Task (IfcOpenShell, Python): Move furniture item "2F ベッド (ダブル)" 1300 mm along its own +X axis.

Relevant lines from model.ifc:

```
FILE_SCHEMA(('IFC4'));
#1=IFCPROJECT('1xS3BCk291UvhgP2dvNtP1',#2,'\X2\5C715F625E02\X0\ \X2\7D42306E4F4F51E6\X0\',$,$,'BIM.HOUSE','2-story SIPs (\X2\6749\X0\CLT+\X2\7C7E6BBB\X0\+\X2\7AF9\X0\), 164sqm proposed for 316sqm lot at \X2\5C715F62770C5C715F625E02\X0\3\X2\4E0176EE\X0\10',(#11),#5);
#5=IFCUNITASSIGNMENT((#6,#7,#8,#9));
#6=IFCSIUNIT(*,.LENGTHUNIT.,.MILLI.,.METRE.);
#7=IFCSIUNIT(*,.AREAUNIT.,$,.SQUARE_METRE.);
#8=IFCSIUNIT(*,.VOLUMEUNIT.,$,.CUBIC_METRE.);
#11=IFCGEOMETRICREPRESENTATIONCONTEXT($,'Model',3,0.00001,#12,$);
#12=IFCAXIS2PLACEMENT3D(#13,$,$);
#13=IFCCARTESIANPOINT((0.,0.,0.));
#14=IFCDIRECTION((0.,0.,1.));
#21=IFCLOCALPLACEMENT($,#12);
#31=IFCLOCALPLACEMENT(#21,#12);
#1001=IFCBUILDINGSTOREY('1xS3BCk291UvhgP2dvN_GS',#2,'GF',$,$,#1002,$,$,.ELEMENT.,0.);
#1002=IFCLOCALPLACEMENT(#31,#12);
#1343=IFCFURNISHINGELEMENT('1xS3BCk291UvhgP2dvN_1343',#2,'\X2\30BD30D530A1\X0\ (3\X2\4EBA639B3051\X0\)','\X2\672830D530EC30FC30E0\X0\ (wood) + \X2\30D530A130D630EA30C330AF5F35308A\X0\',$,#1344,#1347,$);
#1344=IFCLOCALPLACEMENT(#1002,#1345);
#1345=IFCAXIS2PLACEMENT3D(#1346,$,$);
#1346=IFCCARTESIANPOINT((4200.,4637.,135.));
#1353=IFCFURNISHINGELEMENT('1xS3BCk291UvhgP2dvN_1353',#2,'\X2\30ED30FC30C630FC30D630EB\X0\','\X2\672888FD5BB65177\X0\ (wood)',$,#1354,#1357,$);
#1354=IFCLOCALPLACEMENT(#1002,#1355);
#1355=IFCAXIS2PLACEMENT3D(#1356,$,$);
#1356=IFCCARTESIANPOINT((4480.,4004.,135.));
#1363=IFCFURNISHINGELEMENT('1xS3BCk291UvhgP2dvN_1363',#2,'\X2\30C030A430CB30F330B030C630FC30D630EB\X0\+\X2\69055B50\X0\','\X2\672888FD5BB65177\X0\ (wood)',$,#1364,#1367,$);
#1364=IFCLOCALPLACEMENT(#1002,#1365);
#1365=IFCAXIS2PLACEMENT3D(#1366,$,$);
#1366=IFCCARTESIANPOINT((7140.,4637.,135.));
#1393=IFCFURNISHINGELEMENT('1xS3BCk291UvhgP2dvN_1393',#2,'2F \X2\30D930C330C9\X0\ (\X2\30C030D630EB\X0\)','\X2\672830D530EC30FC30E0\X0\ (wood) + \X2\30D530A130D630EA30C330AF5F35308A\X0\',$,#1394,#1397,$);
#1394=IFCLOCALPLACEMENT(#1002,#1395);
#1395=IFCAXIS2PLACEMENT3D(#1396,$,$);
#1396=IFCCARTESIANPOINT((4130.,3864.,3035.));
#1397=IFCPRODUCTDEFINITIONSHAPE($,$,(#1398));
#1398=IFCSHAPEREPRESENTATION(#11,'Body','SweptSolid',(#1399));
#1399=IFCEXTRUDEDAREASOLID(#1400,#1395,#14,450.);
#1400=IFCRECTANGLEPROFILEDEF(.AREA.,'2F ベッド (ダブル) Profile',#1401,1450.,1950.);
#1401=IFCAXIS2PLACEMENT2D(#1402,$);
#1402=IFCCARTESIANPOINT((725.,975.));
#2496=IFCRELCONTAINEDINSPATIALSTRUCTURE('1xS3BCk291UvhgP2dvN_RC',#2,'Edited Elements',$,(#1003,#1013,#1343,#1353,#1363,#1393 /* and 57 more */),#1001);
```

```python
import ifcopenshell
import ifcopenshell.api.geometry
import ifcopenshell.util.placement
import ifcopenshell.util.unit

model = ifcopenshell.open("model.ifc")
unit_scale = ifcopenshell.util.unit.calculate_unit_scale(model)

item = model.by_guid("1xS3BCk291UvhgP2dvN_1393")
matrix = ifcopenshell.util.placement.get_local_placement(item.ObjectPlacement)
matrix[:3, 3] += matrix[:3, 0] * 1.3 / unit_scale
ifcopenshell.api.geometry.edit_object_placement(model, product=item, matrix=matrix, is_si=False)

print(ifcopenshell.util.placement.get_local_placement(item.ObjectPlacement).round(3) + 0.0)

model.write("model_edited.ifc")
```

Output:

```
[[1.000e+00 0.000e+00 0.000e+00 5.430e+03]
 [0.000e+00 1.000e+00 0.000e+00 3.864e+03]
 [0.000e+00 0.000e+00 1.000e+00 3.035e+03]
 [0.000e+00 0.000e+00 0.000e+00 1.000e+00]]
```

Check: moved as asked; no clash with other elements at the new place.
